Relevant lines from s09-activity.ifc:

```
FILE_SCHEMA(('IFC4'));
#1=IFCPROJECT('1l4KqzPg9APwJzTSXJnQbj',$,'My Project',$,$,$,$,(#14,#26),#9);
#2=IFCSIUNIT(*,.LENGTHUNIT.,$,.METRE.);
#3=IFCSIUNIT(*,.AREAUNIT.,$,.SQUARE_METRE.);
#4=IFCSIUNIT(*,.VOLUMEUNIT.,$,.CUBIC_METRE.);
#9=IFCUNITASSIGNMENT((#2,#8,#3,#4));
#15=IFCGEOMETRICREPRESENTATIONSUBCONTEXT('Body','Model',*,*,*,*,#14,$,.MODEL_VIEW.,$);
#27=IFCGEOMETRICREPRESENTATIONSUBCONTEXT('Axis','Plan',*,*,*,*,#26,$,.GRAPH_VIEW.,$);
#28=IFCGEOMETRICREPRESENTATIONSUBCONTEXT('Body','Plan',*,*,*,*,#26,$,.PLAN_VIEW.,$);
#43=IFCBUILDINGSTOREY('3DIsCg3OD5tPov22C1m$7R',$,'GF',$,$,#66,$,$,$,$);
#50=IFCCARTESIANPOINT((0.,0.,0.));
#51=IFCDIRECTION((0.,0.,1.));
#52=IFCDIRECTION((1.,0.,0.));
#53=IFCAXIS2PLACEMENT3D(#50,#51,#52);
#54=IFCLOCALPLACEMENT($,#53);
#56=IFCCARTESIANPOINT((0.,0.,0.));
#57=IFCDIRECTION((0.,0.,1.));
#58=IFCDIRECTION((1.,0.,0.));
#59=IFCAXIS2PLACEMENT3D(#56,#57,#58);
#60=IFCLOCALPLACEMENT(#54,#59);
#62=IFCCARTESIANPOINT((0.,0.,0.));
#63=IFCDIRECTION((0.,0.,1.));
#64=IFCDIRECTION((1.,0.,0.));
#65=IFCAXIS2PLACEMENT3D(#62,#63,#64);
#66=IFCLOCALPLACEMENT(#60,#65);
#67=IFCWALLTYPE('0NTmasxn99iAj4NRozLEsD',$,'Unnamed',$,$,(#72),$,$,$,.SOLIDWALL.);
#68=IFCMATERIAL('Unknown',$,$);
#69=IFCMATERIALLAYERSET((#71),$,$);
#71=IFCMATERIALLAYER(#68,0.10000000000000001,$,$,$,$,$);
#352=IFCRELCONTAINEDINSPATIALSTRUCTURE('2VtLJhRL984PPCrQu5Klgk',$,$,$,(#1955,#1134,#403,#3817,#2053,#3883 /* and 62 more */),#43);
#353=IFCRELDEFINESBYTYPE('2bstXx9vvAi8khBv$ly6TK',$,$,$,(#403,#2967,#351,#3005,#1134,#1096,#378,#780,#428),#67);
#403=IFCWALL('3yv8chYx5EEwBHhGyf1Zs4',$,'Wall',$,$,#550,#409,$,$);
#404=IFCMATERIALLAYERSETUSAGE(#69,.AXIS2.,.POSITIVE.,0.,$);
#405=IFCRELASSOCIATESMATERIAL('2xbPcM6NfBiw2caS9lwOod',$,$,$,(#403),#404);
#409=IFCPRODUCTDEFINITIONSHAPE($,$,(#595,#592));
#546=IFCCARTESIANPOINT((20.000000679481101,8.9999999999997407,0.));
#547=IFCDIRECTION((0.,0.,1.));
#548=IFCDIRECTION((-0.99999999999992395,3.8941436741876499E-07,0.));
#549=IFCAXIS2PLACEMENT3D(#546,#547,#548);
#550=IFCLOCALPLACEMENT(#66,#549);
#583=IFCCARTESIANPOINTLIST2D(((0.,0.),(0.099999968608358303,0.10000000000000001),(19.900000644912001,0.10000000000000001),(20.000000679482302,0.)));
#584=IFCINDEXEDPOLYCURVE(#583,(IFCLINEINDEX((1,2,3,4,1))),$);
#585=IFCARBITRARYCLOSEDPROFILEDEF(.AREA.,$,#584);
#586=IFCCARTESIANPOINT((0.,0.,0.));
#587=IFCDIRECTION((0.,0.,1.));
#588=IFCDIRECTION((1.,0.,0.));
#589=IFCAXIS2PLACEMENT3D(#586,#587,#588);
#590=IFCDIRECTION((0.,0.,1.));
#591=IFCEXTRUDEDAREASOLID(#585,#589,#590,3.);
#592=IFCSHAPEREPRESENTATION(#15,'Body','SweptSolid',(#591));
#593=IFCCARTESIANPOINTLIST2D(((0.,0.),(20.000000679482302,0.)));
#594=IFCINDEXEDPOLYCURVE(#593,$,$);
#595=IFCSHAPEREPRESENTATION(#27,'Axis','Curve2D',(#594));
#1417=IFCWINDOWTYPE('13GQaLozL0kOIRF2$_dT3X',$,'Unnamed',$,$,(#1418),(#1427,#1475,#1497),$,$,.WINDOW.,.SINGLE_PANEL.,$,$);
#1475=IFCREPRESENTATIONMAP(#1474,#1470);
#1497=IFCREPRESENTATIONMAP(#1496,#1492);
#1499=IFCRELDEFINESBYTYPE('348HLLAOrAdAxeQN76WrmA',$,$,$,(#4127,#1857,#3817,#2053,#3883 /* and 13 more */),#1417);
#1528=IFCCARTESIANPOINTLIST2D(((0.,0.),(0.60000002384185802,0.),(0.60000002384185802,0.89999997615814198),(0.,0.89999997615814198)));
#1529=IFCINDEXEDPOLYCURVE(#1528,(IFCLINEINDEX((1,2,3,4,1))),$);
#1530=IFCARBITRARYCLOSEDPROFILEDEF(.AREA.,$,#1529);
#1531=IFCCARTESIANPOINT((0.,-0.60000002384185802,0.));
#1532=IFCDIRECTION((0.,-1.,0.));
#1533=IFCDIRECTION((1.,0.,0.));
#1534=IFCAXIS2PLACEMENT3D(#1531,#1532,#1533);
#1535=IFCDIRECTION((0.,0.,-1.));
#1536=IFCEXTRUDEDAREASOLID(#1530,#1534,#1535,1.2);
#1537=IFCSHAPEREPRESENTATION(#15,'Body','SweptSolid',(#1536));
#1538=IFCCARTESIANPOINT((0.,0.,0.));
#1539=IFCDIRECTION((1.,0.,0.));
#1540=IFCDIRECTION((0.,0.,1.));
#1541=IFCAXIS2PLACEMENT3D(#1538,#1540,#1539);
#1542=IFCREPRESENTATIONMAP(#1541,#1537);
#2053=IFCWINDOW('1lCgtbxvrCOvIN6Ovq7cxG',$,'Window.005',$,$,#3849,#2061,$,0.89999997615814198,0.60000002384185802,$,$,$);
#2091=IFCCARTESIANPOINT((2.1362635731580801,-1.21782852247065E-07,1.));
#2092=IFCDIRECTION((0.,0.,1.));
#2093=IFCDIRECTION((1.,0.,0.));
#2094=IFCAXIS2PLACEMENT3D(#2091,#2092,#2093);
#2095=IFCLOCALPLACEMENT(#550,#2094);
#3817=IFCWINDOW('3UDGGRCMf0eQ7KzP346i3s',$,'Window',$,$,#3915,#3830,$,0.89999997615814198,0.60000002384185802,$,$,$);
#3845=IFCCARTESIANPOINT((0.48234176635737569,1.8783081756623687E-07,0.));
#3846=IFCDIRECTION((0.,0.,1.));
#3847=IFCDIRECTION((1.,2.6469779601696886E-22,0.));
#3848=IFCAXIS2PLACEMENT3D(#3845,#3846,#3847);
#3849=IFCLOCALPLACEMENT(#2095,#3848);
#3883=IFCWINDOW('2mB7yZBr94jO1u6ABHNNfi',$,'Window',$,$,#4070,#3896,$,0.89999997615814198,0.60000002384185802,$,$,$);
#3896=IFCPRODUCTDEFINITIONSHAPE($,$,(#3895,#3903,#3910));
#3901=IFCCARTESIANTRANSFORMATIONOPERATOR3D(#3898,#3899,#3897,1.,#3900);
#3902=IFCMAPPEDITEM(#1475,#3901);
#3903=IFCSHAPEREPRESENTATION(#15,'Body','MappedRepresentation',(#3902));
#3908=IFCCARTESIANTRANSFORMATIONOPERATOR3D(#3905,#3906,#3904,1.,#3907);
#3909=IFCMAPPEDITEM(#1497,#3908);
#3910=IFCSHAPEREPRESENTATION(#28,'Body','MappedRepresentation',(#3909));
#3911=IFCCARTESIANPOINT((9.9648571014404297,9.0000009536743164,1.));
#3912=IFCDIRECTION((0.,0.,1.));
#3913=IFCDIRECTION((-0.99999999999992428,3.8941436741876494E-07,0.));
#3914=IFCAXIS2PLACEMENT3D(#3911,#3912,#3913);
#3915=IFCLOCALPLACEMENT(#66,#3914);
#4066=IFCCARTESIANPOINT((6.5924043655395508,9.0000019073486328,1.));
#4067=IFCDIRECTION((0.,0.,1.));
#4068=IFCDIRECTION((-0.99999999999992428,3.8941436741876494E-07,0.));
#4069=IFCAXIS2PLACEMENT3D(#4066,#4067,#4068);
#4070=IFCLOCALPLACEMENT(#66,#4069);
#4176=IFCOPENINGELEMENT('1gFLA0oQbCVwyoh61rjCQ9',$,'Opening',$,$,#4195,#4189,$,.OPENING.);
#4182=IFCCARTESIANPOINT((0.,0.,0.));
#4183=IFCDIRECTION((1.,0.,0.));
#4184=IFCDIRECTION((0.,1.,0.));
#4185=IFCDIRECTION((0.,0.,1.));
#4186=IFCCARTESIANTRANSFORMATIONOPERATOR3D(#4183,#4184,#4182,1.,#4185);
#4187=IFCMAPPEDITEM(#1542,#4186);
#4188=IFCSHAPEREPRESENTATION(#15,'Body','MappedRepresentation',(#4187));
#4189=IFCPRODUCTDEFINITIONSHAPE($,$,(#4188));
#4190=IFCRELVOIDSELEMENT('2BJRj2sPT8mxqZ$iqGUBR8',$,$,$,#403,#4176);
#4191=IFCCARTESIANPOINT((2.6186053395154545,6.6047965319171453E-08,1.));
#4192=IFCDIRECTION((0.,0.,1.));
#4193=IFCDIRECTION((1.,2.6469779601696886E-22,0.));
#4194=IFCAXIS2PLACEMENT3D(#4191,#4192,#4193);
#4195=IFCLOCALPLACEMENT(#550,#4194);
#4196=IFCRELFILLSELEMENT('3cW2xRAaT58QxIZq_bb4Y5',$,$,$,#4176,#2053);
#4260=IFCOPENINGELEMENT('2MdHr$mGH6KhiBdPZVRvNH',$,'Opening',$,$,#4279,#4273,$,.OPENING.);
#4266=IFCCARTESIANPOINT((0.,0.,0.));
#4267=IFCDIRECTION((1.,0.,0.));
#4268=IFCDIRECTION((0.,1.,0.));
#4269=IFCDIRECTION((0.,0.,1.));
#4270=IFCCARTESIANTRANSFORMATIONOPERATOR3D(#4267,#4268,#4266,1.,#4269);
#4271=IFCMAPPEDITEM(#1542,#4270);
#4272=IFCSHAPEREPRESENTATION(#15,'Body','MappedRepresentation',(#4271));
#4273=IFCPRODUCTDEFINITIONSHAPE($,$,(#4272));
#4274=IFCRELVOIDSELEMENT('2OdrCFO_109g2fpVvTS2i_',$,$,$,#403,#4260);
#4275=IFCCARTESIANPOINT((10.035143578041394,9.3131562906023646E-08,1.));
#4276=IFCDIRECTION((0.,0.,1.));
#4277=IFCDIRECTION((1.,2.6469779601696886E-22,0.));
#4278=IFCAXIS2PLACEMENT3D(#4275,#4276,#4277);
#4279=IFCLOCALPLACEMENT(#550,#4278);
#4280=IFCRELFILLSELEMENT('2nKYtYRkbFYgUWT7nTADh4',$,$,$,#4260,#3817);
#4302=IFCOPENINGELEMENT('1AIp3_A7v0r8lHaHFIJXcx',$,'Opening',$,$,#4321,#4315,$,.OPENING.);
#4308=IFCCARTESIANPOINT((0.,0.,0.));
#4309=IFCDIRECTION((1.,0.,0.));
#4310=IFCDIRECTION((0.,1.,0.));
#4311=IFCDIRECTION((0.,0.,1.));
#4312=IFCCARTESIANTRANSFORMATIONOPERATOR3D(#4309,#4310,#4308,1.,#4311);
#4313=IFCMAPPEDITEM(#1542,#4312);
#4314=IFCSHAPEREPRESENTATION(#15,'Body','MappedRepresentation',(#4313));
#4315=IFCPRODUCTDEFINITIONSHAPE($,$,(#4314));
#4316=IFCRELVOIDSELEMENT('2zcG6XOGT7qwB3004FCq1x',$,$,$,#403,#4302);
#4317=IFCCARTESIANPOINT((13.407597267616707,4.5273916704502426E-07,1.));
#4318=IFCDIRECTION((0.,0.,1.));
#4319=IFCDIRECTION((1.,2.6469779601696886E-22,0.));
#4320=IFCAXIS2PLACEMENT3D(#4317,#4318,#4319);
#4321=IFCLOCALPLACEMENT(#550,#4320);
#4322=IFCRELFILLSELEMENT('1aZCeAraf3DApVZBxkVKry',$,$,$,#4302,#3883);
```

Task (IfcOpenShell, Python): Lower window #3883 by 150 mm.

```python
import numpy as np
import ifcopenshell
import ifcopenshell.api.geometry
import ifcopenshell.util.placement
import ifcopenshell.util.unit

model = ifcopenshell.open("s09-activity.ifc")
unit_scale = ifcopenshell.util.unit.calculate_unit_scale(model)

window = model.by_guid("2mB7yZBr94jO1u6ABHNNfi")
opening = window.FillsVoids[0].RelatingOpeningElement
dz = -0.15

shift = np.array([0.0, 0.0, dz])
# The window is not placed relative to its opening, so move both.
for product in (opening, window):
    matrix = ifcopenshell.util.placement.get_local_placement(product.ObjectPlacement)
    matrix[:3, 3] += shift
    ifcopenshell.api.geometry.edit_object_placement(model, product=product, matrix=matrix, is_si=False)

print(f"moved by {dz * unit_scale:+.3f} m")

model.write("s09-activity_updated.ifc")
```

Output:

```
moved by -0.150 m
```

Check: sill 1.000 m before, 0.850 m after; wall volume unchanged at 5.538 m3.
